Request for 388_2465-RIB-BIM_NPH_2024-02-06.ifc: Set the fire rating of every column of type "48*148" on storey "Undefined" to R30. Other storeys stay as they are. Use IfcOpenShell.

First a look at what the model holds.

```python
import ifcopenshell
import ifcopenshell.util.element

model = ifcopenshell.open("388_2465-RIB-BIM_NPH_2024-02-06.ifc")
print(model.schema)
storey = next(s for s in model.by_type("IfcBuildingStorey") if s.Name == "Undefined")
columns = [e for e in ifcopenshell.util.element.get_decomposition(storey) if e.is_a("IfcColumn")]
seen = {}
for e in columns:
    element_type = ifcopenshell.util.element.get_type(e)
    key = (element_type.Name if element_type != e and element_type else None, ifcopenshell.util.element.get_pset(e, "Pset_ColumnCommon", "FireRating"))
    seen[key] = seen.get(key, 0) + 1
for (name, value), count in sorted(seen.items(), key=str):
    print(count, "x", name, "|", value)
```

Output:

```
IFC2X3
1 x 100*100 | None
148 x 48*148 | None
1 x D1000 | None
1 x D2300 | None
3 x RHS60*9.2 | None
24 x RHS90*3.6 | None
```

```python
import ifcopenshell
import ifcopenshell.api.pset
import ifcopenshell.util.element

model = ifcopenshell.open("388_2465-RIB-BIM_NPH_2024-02-06.ifc")

storey = next(s for s in model.by_type("IfcBuildingStorey") if s.Name == "Undefined")
columns = [e for e in ifcopenshell.util.element.get_decomposition(storey) if e.is_a("IfcColumn")]

count = 0
for e in columns:
    element_type = ifcopenshell.util.element.get_type(e)
    if element_type in (None, e) or element_type.Name != "48*148":
        continue
    found = ifcopenshell.util.element.get_pset(e, "Pset_ColumnCommon", should_inherit=False)
    if found:
        pset = model.by_id(found["id"])
        if len(ifcopenshell.util.element.get_elements_by_pset(pset)) > 1:
            pset = ifcopenshell.api.pset.unshare_pset(model, products=[e], pset=pset)[0]
    else:
        pset = ifcopenshell.api.pset.add_pset(model, product=e, name="Pset_ColumnCommon")
    ifcopenshell.api.pset.edit_pset(model, pset=pset, properties={"FireRating": "R30"})
    count += 1

print(count, "columns updated")

model.write("388_2465-RIB-BIM_NPH_2024-02-06_edited.ifc")
```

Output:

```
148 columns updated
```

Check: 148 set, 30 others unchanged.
